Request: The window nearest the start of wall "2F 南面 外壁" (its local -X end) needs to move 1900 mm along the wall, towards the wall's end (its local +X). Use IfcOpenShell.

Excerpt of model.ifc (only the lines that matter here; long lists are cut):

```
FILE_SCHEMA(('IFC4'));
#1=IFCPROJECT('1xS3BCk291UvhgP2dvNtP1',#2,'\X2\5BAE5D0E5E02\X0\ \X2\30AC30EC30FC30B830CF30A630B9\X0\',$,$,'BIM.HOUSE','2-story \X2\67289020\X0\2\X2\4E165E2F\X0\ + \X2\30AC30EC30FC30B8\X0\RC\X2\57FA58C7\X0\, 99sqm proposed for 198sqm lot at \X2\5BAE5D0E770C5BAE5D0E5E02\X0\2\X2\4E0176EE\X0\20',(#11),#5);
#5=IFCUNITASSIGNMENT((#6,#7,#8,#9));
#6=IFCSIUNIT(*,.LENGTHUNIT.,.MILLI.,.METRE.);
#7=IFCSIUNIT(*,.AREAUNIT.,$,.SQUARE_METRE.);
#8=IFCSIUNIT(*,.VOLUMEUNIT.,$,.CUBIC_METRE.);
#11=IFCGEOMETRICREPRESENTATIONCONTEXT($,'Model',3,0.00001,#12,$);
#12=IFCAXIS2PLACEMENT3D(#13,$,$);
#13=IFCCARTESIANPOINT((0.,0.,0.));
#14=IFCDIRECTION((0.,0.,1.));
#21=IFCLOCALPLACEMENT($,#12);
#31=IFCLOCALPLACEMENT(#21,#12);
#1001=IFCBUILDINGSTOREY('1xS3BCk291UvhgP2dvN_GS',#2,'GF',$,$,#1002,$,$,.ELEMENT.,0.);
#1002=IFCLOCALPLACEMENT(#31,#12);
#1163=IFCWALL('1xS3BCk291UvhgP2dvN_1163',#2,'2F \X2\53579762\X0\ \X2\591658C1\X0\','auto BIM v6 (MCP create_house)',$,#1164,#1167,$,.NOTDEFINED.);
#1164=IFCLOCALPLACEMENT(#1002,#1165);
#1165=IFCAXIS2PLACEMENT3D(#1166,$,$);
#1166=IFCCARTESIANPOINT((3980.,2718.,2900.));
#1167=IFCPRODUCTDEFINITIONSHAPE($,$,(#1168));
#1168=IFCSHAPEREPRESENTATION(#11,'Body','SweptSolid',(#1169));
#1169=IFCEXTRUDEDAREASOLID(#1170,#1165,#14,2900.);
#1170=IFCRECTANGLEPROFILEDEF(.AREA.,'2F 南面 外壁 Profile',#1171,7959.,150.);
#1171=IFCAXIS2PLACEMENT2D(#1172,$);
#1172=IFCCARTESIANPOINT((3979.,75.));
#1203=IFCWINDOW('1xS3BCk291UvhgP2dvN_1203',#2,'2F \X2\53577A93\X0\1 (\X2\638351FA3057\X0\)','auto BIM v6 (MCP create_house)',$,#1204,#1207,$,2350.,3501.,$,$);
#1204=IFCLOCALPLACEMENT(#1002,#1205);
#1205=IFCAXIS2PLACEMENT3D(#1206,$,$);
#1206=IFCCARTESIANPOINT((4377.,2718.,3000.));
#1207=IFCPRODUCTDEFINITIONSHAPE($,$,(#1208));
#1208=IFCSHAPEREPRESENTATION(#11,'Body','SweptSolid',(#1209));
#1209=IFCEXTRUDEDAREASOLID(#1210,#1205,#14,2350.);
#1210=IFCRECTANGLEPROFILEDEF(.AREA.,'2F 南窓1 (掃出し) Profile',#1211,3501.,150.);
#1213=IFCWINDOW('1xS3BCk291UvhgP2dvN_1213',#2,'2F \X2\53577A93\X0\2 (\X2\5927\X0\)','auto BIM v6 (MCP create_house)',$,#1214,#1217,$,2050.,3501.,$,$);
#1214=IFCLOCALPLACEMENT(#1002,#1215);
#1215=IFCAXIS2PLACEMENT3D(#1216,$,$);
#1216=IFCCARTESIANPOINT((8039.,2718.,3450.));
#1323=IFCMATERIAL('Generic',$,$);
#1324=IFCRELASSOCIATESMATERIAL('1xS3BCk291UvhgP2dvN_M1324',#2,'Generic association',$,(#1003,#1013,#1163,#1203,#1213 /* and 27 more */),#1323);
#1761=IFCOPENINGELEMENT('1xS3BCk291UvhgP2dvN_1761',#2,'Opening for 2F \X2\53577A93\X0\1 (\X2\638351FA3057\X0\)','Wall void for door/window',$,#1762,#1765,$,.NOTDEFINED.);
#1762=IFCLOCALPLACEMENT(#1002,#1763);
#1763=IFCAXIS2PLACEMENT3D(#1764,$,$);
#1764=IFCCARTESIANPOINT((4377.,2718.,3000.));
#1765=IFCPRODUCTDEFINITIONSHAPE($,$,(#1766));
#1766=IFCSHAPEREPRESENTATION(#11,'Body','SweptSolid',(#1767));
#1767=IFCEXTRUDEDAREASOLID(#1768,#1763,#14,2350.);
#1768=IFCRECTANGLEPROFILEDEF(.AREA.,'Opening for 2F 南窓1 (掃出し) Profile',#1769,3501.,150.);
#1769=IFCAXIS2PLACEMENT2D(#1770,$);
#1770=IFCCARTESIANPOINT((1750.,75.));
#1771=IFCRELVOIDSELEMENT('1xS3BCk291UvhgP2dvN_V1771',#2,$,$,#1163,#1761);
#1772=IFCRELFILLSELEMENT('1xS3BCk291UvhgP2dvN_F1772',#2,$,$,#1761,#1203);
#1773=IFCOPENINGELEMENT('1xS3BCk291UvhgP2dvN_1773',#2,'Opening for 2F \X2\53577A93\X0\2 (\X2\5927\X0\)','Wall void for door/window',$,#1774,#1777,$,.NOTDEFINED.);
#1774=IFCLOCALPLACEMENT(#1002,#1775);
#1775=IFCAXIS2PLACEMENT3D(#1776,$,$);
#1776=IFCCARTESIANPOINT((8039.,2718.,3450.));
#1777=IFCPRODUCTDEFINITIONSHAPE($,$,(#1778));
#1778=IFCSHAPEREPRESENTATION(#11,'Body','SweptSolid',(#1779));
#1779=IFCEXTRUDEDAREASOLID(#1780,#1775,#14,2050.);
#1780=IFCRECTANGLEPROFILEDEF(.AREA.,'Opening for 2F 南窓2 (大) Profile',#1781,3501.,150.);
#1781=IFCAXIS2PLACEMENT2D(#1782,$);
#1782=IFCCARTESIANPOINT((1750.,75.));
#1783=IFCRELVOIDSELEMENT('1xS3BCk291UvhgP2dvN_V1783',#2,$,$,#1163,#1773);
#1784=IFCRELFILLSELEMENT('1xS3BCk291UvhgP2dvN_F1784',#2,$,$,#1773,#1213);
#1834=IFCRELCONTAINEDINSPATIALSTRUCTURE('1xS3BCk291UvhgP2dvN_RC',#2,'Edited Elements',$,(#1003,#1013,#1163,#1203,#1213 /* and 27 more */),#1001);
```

```python
import ifcopenshell
import ifcopenshell.api.geometry
import ifcopenshell.util.placement
import ifcopenshell.util.unit

model = ifcopenshell.open("model.ifc")
unit_scale = ifcopenshell.util.unit.calculate_unit_scale(model)

window = model.by_guid("1xS3BCk291UvhgP2dvN_1203")
opening = window.FillsVoids[0].RelatingOpeningElement
wall = opening.VoidsElements[0].RelatingBuildingElement

wall_matrix = ifcopenshell.util.placement.get_local_placement(wall.ObjectPlacement)
shift = wall_matrix[:3, 0] * 1.9 / unit_scale
before = ifcopenshell.util.placement.get_local_placement(window.ObjectPlacement)[:3, 3].copy()

# The window is not placed relative to its opening, so move both.
for product in (opening, window):
    matrix = ifcopenshell.util.placement.get_local_placement(product.ObjectPlacement)
    matrix[:3, 3] += shift
    ifcopenshell.api.geometry.edit_object_placement(model, product=product, matrix=matrix, is_si=False)

after = ifcopenshell.util.placement.get_local_placement(window.ObjectPlacement)[:3, 3]
print("window moved by", (after - before).round(3) + 0.0)

model.write("model_updated.ifc")
```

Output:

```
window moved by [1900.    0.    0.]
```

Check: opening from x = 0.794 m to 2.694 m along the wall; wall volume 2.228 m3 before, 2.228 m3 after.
